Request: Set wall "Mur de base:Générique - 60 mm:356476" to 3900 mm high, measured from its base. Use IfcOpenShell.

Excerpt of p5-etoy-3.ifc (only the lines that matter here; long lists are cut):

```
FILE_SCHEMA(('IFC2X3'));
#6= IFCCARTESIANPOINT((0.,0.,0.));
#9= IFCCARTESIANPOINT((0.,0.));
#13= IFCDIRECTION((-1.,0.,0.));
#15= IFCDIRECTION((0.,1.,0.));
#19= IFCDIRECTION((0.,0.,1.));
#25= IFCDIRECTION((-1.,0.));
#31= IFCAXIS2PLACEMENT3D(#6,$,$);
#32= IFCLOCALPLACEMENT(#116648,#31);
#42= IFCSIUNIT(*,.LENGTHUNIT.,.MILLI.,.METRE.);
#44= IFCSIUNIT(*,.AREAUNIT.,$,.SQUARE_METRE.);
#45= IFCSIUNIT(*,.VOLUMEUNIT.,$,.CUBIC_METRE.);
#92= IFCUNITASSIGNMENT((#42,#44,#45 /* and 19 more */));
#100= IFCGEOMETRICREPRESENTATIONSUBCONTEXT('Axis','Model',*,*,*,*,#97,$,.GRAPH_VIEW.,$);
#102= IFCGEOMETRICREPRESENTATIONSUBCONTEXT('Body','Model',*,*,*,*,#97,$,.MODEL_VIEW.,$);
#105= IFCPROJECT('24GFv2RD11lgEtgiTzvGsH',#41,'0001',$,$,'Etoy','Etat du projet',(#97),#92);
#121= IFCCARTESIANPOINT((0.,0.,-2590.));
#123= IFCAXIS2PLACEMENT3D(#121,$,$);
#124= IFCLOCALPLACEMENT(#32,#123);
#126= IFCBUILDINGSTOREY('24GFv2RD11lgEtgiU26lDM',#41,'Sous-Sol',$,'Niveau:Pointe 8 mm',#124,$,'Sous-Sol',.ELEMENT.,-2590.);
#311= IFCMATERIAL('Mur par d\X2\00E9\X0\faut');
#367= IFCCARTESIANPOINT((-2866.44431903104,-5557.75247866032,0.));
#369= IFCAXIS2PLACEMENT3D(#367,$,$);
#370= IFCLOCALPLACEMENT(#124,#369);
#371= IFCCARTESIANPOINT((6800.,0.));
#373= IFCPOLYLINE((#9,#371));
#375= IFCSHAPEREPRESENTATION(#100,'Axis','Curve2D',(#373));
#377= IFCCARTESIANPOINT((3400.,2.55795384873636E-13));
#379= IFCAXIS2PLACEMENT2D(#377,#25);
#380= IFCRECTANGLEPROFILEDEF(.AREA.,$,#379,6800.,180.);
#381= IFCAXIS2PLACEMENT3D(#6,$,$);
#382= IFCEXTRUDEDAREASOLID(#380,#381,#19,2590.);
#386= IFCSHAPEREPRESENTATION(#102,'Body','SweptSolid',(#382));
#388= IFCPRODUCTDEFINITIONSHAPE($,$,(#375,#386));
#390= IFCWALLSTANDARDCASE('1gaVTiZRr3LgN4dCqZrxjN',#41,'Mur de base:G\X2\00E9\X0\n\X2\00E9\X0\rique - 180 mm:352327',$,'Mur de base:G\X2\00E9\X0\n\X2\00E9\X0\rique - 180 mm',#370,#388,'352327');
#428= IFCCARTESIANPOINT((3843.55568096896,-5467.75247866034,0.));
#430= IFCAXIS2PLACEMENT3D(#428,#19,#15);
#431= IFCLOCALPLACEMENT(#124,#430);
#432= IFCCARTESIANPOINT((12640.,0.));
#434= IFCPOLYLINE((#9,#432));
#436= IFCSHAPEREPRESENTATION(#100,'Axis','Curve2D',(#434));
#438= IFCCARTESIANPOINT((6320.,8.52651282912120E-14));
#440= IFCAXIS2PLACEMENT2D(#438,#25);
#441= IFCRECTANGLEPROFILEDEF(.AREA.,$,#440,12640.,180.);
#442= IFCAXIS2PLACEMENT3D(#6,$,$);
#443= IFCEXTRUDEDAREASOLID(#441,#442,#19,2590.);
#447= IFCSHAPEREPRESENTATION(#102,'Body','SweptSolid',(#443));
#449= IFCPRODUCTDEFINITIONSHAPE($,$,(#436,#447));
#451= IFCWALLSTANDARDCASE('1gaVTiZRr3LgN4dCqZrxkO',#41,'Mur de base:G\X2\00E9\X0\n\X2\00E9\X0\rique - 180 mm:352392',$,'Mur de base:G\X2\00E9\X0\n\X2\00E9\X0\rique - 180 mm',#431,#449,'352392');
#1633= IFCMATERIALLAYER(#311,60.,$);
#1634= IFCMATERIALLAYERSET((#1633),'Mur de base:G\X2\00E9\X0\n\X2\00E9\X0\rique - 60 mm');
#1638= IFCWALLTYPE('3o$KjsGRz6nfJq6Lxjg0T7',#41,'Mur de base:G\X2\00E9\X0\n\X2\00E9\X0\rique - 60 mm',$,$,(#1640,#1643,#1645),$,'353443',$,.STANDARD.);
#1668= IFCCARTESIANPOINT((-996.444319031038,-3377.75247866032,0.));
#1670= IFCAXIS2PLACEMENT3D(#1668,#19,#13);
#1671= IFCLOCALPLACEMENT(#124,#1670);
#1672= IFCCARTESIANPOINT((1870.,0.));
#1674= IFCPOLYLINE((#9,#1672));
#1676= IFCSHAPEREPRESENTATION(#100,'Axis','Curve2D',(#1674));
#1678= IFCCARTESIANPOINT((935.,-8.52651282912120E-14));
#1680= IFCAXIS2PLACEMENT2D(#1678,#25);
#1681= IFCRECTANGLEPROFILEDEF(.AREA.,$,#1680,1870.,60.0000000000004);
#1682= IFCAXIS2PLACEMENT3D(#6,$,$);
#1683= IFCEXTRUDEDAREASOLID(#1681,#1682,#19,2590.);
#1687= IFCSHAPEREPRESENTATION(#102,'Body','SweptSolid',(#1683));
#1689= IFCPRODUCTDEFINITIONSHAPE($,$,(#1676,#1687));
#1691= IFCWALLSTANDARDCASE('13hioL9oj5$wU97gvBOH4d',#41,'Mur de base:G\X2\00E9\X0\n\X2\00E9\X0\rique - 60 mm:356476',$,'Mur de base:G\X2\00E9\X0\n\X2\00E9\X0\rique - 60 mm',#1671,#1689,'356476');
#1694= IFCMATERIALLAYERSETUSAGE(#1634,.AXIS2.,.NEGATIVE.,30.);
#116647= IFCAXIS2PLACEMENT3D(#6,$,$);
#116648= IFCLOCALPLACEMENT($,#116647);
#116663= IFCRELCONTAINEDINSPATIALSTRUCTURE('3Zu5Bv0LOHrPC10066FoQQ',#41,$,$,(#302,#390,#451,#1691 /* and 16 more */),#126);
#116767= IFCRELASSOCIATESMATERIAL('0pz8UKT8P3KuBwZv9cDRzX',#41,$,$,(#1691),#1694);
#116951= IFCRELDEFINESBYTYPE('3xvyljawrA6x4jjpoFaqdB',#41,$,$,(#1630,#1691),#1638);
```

```python
import ifcopenshell
import ifcopenshell.geom
import ifcopenshell.util.representation
import ifcopenshell.util.shape

model = ifcopenshell.open("p5-etoy-3.ifc")
settings = ifcopenshell.geom.settings()


def volume(element):
    """Net volume in cubic metres, openings subtracted."""
    shape = ifcopenshell.geom.create_shape(settings, element)
    return ifcopenshell.util.shape.get_volume(shape.geometry)


wall = model.by_id(1691)
before = volume(wall)

body = ifcopenshell.util.representation.get_representation(wall, "Model", "Body")
solid = body.Items[0]
old_height = solid.Depth
solid.Depth = 3900.0
after = volume(wall)

print(f"height {old_height:g} -> {solid.Depth:g}, volume {before:.3f} -> {after:.3f} m3")

model.write("p5-etoy-3_updated.ifc")
```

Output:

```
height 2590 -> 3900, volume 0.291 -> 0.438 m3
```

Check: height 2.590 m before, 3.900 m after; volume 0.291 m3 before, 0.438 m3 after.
